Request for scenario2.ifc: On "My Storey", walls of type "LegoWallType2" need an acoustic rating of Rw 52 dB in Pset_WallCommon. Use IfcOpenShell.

First a look at what the model holds.

```python
import ifcopenshell
import ifcopenshell.util.element

model = ifcopenshell.open("scenario2.ifc")
print(model.schema)
storey = next(s for s in model.by_type("IfcBuildingStorey") if s.Name == "My Storey")
walls = [e for e in ifcopenshell.util.element.get_decomposition(storey) if e.is_a("IfcWall")]
seen = {}
for e in walls:
    element_type = ifcopenshell.util.element.get_type(e)
    key = (element_type.Name if element_type != e and element_type else None, ifcopenshell.util.element.get_pset(e, "Pset_WallCommon", "AcousticRating"))
    seen[key] = seen.get(key, 0) + 1
for (name, value), count in sorted(seen.items(), key=str):
    print(count, "x", name, "|", value)
```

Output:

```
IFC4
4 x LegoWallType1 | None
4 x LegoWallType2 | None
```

```python
import ifcopenshell
import ifcopenshell.api.pset
import ifcopenshell.util.element

model = ifcopenshell.open("scenario2.ifc")

storey = next(s for s in model.by_type("IfcBuildingStorey") if s.Name == "My Storey")
walls = [e for e in ifcopenshell.util.element.get_decomposition(storey) if e.is_a("IfcWall")]

count = 0
for e in walls:
    element_type = ifcopenshell.util.element.get_type(e)
    if element_type in (None, e) or element_type.Name != "LegoWallType2":
        continue
    # add_pset returns the element's existing set when there is one.
    pset = ifcopenshell.api.pset.add_pset(model, product=e, name="Pset_WallCommon")
    ifcopenshell.api.pset.edit_pset(model, pset=pset, properties={"AcousticRating": "Rw 52 dB"})
    count += 1

print(count, "walls updated")

model.write("scenario2_updated.ifc")
```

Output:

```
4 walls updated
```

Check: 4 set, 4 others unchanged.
